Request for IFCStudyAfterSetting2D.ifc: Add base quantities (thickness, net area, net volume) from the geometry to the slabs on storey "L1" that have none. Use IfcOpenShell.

First a look at what the model holds.

```python
import ifcopenshell
import ifcopenshell.util.element
import ifcopenshell.util.unit

model = ifcopenshell.open("IFCStudyAfterSetting2D.ifc")
print(model.schema)
for unit_type in ("LENGTHUNIT", "AREAUNIT", "VOLUMEUNIT"):
    print(unit_type, ifcopenshell.util.unit.calculate_unit_scale(model, unit_type))
storey = next(s for s in model.by_type("IfcBuildingStorey") if s.Name == "L1")
slabs = [e for e in ifcopenshell.util.element.get_decomposition(storey) if e.is_a("IfcSlab")]
for e in sorted(slabs, key=lambda e: e.id()):
    print(e.id(), e.is_a(), e.Name, list(ifcopenshell.util.element.get_psets(e, qtos_only=True)), sep=" | ")
```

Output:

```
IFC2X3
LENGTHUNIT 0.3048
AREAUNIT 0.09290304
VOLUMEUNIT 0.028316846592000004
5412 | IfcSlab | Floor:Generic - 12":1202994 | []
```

```python
import ifcopenshell
import ifcopenshell.api.pset
import ifcopenshell.geom
import ifcopenshell.util.element
import ifcopenshell.util.shape
import ifcopenshell.util.unit

model = ifcopenshell.open("IFCStudyAfterSetting2D.ifc")
unit_scale = ifcopenshell.util.unit.calculate_unit_scale(model)
area_scale = ifcopenshell.util.unit.calculate_unit_scale(model, "AREAUNIT")
volume_scale = ifcopenshell.util.unit.calculate_unit_scale(model, "VOLUMEUNIT")
settings = ifcopenshell.geom.settings()

storey = next(s for s in model.by_type("IfcBuildingStorey") if s.Name == "L1")
slabs = [e for e in ifcopenshell.util.element.get_decomposition(storey) if e.is_a("IfcSlab")]

for e in sorted(slabs, key=lambda e: e.id()):
    if ifcopenshell.util.element.get_psets(e, qtos_only=True, should_inherit=False):
        continue
    # Geometry comes back in metres, in the element's own axes.
    shape = ifcopenshell.geom.create_shape(settings, e)
    values = {
        "Width": ifcopenshell.util.shape.get_z(shape.geometry) / unit_scale,
        "NetArea": ifcopenshell.util.shape.get_footprint_area(shape.geometry) / area_scale,
        "NetVolume": ifcopenshell.util.shape.get_volume(shape.geometry) / volume_scale,
    }
    qto = ifcopenshell.api.pset.add_qto(model, product=e, name="BaseQuantities")
    ifcopenshell.api.pset.edit_qto(model, qto=qto, properties=values)
    print(e.id(), {k: round(v, 3) for k, v in values.items()})

model.write("IFCStudyAfterSetting2D_v2.ifc")
```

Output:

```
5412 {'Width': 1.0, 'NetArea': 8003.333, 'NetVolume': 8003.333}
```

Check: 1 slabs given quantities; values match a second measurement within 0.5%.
